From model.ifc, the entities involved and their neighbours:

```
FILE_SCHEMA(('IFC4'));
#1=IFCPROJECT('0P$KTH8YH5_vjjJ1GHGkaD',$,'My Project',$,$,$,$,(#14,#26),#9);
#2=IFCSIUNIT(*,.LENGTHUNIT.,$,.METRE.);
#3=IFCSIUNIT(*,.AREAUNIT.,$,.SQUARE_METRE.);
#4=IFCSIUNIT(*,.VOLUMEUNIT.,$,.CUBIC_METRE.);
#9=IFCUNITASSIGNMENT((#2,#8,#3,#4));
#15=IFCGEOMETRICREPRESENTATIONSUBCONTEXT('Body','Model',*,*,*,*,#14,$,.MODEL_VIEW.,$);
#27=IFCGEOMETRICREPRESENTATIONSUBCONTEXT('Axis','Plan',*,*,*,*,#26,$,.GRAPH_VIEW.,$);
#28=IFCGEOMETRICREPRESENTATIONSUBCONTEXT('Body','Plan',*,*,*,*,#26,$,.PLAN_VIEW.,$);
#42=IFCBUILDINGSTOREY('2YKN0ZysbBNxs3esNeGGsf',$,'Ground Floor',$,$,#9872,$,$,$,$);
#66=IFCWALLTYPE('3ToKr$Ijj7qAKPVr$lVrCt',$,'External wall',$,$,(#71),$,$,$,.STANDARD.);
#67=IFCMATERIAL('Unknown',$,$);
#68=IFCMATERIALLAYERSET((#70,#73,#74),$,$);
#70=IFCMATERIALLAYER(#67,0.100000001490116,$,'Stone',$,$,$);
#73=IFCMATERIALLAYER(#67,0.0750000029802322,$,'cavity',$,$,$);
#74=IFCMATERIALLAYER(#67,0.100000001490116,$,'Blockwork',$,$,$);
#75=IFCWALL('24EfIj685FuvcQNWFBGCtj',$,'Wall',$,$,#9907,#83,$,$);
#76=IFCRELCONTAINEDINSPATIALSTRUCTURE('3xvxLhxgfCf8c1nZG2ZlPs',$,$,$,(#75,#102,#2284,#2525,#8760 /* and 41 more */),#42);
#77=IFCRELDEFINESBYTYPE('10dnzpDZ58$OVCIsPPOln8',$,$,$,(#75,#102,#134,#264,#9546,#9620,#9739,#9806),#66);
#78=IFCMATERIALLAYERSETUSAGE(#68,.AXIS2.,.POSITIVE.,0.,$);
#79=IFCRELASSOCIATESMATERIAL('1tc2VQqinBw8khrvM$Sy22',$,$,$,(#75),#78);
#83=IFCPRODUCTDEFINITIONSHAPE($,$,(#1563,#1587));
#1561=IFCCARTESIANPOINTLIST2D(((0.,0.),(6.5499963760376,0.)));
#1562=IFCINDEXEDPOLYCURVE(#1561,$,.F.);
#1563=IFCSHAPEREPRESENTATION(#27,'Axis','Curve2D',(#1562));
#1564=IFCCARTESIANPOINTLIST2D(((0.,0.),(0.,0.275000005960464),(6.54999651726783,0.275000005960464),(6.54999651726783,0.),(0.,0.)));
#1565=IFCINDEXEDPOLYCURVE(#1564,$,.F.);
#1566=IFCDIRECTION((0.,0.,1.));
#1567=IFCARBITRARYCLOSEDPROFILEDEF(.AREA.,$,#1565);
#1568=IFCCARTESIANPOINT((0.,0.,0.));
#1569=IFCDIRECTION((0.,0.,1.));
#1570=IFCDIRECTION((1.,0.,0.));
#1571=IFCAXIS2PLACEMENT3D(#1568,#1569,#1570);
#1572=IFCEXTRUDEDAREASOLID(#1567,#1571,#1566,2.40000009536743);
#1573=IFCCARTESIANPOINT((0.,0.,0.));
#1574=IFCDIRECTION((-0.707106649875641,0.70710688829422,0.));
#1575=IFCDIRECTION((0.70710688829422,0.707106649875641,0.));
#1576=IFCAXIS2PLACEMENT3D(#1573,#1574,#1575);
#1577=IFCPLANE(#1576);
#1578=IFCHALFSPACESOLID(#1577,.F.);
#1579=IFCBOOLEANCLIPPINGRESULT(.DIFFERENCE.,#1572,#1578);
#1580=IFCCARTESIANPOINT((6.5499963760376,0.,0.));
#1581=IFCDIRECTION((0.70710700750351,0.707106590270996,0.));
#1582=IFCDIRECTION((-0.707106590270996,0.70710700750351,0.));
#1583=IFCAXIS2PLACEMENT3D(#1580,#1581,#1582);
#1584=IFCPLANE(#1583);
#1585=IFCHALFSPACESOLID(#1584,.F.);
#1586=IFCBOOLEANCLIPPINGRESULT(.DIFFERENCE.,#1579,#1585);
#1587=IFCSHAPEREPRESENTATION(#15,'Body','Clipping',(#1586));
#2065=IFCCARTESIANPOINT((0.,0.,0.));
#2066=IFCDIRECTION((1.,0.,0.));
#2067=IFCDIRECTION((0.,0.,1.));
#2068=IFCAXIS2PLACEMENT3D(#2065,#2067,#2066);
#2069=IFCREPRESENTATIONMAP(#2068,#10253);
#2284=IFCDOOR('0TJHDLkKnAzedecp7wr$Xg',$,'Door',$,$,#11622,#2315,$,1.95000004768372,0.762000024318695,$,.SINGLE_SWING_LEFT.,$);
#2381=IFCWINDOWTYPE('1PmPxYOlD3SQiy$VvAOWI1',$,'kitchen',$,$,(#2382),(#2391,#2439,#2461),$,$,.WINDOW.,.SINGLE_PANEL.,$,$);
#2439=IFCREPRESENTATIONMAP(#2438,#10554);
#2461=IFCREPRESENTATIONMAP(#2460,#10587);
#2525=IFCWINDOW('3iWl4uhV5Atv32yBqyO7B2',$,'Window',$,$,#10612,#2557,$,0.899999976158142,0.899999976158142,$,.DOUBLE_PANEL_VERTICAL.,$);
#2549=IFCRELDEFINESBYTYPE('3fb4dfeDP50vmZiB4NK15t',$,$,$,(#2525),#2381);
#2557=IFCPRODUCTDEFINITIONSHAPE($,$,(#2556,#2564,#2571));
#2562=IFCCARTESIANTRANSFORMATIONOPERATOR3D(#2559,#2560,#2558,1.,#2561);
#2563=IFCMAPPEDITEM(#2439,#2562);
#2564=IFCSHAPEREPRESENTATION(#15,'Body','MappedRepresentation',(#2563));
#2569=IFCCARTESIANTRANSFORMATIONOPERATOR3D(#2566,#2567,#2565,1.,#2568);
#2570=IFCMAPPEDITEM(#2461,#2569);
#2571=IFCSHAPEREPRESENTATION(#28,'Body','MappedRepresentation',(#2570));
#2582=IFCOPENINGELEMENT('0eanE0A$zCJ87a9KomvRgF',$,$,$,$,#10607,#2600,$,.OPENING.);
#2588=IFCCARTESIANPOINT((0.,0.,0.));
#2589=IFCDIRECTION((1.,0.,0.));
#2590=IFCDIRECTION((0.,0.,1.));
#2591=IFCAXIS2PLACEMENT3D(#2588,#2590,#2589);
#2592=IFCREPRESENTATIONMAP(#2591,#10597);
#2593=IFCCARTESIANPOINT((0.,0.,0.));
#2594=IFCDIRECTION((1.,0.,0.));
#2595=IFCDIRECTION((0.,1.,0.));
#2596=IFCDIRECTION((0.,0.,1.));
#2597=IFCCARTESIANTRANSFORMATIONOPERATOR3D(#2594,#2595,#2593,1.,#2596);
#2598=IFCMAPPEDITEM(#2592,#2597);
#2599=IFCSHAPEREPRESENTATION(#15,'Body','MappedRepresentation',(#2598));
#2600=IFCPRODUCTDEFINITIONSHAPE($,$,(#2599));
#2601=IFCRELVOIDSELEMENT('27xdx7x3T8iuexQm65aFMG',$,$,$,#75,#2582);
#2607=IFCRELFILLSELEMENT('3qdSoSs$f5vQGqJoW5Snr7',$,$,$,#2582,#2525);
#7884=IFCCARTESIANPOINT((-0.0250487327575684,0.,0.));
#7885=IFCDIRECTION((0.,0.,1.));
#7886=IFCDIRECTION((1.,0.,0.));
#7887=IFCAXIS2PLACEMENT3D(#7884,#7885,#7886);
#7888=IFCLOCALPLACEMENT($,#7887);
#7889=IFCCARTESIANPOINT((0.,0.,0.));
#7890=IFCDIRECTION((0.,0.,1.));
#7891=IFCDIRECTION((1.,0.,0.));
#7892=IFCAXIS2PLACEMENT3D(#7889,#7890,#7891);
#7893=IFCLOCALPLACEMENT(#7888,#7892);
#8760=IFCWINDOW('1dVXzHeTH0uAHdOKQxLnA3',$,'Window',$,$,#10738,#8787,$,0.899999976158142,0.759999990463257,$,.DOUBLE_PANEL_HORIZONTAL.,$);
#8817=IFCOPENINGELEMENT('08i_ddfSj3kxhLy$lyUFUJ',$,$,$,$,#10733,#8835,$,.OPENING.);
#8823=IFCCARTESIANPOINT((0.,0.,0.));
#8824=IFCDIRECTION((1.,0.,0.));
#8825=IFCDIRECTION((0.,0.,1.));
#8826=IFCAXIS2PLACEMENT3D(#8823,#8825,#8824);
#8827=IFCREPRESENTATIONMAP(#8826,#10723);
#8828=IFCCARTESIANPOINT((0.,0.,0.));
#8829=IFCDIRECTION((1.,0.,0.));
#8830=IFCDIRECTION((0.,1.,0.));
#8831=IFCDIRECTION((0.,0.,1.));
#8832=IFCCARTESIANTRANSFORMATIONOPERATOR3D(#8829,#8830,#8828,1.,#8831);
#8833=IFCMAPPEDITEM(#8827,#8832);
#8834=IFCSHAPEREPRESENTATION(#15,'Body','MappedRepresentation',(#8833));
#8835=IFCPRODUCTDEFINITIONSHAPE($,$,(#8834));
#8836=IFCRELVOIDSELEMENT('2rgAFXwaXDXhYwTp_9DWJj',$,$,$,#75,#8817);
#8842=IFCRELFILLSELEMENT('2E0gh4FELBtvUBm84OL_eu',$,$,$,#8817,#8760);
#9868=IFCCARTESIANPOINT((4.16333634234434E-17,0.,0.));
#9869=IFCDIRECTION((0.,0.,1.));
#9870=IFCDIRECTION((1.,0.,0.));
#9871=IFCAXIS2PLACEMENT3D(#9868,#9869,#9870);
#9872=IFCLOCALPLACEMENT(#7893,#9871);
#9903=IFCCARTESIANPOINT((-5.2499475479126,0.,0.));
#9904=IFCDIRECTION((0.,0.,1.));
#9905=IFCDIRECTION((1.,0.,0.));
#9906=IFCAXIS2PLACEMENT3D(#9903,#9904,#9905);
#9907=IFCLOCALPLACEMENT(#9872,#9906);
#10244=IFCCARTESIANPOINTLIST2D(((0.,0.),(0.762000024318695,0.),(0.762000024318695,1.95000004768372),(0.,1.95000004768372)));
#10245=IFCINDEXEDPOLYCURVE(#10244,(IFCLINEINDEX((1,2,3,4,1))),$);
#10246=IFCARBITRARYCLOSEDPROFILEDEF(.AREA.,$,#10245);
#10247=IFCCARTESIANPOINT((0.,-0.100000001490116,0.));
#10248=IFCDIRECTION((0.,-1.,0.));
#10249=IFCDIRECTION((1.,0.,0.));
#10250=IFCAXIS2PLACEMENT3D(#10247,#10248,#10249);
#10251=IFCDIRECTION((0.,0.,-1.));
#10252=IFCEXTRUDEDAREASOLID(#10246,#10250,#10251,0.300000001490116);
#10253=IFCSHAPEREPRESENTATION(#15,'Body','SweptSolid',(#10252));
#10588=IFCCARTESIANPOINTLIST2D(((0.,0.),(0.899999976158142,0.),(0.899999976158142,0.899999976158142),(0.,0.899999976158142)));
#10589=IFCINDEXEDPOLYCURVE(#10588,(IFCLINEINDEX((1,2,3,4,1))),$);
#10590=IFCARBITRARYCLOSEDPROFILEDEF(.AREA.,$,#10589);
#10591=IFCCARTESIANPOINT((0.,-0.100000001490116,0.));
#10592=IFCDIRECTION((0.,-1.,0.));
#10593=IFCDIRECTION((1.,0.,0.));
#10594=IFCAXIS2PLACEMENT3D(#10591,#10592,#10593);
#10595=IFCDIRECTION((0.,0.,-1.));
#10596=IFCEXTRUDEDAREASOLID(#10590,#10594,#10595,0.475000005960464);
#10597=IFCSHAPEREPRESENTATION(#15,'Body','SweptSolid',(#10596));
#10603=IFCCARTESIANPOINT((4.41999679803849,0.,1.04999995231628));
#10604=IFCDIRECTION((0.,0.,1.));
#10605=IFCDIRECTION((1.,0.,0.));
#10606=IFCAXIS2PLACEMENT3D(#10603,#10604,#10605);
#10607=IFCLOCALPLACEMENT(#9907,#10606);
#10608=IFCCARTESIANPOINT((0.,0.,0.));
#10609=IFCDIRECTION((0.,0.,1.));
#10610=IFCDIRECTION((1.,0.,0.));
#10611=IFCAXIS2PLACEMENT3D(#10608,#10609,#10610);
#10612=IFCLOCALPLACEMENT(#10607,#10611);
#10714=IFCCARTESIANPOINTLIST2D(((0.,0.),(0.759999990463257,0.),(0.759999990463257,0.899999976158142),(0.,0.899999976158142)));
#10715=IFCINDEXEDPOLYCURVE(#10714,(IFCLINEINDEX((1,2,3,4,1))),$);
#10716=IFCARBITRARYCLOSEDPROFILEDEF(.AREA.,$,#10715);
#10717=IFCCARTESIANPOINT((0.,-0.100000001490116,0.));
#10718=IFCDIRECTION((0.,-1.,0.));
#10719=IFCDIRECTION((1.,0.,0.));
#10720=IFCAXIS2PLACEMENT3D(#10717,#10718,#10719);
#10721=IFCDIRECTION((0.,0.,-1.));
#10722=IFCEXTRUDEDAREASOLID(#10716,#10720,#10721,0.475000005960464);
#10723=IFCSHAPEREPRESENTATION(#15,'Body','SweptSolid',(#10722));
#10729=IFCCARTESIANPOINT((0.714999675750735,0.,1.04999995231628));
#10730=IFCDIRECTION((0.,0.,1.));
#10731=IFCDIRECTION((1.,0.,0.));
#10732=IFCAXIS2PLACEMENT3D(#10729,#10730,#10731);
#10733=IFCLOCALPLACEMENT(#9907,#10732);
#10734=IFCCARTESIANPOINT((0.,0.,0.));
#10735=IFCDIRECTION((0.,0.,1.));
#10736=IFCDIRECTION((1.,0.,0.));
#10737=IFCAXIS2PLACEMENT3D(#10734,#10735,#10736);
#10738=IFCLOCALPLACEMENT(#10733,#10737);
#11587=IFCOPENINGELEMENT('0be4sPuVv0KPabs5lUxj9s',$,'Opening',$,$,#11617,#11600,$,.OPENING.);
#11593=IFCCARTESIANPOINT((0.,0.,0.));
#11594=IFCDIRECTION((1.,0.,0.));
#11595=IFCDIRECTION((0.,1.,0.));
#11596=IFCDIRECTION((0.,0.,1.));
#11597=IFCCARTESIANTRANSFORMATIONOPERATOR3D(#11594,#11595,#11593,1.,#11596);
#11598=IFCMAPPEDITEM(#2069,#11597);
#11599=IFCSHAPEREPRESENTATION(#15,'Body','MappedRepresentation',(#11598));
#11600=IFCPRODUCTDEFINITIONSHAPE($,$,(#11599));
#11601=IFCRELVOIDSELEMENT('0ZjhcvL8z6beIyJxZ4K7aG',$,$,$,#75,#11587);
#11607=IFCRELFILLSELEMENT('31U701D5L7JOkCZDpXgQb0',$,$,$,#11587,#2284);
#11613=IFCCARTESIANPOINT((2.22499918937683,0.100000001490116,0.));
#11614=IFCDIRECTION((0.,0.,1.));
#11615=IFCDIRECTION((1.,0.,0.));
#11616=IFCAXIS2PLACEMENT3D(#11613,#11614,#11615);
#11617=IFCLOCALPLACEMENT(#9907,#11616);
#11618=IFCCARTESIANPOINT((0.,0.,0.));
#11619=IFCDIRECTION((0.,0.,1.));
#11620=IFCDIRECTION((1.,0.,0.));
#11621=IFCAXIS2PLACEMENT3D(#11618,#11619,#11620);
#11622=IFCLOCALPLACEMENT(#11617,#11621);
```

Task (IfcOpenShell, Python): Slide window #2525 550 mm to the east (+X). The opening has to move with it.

```python
import ifcopenshell
import ifcopenshell.api.geometry
import ifcopenshell.util.placement

model = ifcopenshell.open("model.ifc")

window = model.by_id(2525)
opening = window.FillsVoids[0].RelatingOpeningElement
wall = opening.VoidsElements[0].RelatingBuildingElement

wall_matrix = ifcopenshell.util.placement.get_local_placement(wall.ObjectPlacement)
shift = wall_matrix[:3, 0] * 0.55
before = ifcopenshell.util.placement.get_local_placement(window.ObjectPlacement)[:3, 3].copy()

# The window is placed relative to its opening, so it follows when the opening moves.
matrix = ifcopenshell.util.placement.get_local_placement(opening.ObjectPlacement)
matrix[:3, 3] += shift
ifcopenshell.api.geometry.edit_object_placement(
    model, product=opening, matrix=matrix, is_si=False, should_transform_children=True
)

after = ifcopenshell.util.placement.get_local_placement(window.ObjectPlacement)[:3, 3]
print("window moved by", (after - before).round(3) + 0.0)

model.write("model-out.ifc")
```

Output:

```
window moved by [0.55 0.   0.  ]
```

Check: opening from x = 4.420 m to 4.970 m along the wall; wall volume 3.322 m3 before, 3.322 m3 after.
